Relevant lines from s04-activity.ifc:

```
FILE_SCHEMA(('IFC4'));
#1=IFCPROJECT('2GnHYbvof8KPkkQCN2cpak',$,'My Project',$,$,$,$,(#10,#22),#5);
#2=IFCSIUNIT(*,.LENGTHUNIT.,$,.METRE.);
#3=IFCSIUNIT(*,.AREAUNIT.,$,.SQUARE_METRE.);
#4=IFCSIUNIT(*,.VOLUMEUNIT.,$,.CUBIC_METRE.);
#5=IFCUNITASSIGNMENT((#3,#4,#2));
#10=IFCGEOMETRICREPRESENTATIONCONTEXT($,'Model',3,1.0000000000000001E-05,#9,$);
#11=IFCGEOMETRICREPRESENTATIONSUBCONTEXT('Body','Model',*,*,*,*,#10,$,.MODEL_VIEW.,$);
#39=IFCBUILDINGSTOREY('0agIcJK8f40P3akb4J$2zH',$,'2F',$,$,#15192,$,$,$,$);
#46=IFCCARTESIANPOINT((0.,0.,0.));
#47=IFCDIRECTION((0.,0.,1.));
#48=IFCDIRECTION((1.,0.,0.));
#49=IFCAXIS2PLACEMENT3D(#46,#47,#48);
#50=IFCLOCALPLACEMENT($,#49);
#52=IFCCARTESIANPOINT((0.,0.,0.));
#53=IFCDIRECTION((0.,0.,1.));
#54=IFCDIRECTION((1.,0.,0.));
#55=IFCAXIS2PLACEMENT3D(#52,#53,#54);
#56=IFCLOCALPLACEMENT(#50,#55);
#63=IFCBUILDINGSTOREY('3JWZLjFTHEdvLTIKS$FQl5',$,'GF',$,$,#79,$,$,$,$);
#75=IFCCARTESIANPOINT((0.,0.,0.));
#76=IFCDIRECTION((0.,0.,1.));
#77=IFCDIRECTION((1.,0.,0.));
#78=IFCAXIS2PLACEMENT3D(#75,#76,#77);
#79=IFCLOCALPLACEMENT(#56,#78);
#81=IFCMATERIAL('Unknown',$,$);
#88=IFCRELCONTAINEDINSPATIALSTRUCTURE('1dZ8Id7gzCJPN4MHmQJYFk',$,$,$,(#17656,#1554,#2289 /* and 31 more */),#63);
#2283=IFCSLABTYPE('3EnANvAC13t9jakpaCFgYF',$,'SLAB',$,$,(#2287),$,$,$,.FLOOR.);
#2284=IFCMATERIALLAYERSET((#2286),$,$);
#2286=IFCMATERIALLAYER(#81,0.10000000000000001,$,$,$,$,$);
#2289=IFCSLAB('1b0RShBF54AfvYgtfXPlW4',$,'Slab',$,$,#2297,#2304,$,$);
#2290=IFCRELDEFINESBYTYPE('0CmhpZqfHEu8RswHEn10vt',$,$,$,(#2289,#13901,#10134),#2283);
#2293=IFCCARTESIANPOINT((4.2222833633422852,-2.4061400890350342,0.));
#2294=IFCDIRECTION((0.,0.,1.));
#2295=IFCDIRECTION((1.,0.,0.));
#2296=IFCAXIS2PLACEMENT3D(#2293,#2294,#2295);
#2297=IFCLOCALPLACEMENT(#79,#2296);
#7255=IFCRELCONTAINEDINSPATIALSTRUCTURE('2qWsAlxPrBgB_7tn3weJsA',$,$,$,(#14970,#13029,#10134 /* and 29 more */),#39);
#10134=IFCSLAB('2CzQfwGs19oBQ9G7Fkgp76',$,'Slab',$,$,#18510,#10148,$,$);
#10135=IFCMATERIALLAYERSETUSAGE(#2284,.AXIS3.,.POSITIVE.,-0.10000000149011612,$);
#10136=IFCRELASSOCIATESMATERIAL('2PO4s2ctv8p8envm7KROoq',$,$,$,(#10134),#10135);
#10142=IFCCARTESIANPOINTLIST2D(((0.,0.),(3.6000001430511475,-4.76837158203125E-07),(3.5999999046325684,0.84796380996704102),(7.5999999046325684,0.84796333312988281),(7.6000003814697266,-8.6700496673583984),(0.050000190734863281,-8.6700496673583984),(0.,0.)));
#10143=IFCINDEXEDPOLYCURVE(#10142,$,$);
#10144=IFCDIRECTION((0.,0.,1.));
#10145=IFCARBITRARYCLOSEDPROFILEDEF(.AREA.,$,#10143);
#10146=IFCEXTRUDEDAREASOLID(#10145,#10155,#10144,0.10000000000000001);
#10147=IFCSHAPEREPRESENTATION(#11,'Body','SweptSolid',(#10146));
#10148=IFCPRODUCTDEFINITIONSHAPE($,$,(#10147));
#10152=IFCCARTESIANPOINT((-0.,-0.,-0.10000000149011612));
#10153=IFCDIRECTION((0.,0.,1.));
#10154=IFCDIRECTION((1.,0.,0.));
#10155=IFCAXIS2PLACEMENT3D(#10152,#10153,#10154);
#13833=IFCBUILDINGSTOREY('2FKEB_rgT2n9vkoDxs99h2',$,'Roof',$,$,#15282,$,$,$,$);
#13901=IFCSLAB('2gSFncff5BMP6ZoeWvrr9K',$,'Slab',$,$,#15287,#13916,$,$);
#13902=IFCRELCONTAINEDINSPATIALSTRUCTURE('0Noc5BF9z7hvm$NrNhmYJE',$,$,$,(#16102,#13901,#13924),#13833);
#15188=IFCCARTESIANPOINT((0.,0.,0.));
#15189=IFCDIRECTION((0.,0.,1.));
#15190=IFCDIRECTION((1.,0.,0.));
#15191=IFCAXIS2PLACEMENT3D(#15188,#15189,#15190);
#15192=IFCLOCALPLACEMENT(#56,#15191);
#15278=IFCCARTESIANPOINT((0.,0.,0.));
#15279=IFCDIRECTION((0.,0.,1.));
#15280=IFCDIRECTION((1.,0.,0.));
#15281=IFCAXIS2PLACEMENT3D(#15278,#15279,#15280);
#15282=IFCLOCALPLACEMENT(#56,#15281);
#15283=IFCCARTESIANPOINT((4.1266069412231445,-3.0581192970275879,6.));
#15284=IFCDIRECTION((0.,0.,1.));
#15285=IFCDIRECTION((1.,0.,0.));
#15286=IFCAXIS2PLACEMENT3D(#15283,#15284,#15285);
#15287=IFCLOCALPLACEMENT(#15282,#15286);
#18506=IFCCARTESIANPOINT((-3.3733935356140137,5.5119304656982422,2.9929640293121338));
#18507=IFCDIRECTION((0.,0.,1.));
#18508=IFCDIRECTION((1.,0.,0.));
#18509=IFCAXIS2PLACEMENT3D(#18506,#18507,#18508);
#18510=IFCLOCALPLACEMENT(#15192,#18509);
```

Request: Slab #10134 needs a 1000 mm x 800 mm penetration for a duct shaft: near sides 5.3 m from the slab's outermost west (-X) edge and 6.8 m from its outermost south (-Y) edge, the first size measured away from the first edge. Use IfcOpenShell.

```python
import numpy as np
import ifcopenshell
import ifcopenshell.api.feature
import ifcopenshell.api.geometry
import ifcopenshell.api.root
import ifcopenshell.geom
import ifcopenshell.util.placement
import ifcopenshell.util.representation
import ifcopenshell.util.shape
import ifcopenshell.util.unit

model = ifcopenshell.open("s04-activity.ifc")
unit_scale = ifcopenshell.util.unit.calculate_unit_scale(model)
settings = ifcopenshell.geom.settings()


def volume(element):
    """Net volume in cubic metres, openings subtracted."""
    shape = ifcopenshell.geom.create_shape(settings, element)
    return ifcopenshell.util.shape.get_volume(shape.geometry)


slab = model.by_id(10134)
before = volume(slab)

# Extent in the slab's own axes, in metres. The edges named are its -X and -Y sides.
slab_shape = ifcopenshell.geom.create_shape(settings, slab)
vertices = ifcopenshell.util.shape.get_vertices(slab_shape.geometry)
x_min, y_min, bottom = vertices.min(axis=0)
top = vertices[:, 2].max()

opening = ifcopenshell.api.root.create_entity(model, ifc_class="IfcOpeningElement", name="Duct shaft opening", predefined_type="OPENING")
context = ifcopenshell.util.representation.get_context(model, "Model", "Body", "MODEL_VIEW")
width, depth = 1, 0.8
outline = [(0.0, 0.0), (width, 0.0), (width, depth), (0.0, depth), (0.0, 0.0)]
# Overshoot both faces by 50 mm so the cut is clean.
shape = ifcopenshell.api.geometry.add_slab_representation(
    model, context=context, depth=top - bottom + 0.1, polyline=outline
)
ifcopenshell.api.geometry.assign_representation(model, product=opening, representation=shape)

matrix = ifcopenshell.util.placement.get_local_placement(slab.ObjectPlacement)
matrix[:, 3] = matrix @ np.append(np.array([x_min + 5.3, y_min + 6.8, bottom - 0.05]) / unit_scale, 1.0)
ifcopenshell.api.geometry.edit_object_placement(model, product=opening, matrix=matrix, is_si=False)
ifcopenshell.api.feature.add_feature(model, feature=opening, element=slab)

after = volume(slab)

print(f"slab volume {before:.3f} -> {after:.3f} m3")

model.write("s04-activity_rev.ifc")
```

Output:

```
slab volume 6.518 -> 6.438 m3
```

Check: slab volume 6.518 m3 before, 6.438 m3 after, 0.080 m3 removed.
